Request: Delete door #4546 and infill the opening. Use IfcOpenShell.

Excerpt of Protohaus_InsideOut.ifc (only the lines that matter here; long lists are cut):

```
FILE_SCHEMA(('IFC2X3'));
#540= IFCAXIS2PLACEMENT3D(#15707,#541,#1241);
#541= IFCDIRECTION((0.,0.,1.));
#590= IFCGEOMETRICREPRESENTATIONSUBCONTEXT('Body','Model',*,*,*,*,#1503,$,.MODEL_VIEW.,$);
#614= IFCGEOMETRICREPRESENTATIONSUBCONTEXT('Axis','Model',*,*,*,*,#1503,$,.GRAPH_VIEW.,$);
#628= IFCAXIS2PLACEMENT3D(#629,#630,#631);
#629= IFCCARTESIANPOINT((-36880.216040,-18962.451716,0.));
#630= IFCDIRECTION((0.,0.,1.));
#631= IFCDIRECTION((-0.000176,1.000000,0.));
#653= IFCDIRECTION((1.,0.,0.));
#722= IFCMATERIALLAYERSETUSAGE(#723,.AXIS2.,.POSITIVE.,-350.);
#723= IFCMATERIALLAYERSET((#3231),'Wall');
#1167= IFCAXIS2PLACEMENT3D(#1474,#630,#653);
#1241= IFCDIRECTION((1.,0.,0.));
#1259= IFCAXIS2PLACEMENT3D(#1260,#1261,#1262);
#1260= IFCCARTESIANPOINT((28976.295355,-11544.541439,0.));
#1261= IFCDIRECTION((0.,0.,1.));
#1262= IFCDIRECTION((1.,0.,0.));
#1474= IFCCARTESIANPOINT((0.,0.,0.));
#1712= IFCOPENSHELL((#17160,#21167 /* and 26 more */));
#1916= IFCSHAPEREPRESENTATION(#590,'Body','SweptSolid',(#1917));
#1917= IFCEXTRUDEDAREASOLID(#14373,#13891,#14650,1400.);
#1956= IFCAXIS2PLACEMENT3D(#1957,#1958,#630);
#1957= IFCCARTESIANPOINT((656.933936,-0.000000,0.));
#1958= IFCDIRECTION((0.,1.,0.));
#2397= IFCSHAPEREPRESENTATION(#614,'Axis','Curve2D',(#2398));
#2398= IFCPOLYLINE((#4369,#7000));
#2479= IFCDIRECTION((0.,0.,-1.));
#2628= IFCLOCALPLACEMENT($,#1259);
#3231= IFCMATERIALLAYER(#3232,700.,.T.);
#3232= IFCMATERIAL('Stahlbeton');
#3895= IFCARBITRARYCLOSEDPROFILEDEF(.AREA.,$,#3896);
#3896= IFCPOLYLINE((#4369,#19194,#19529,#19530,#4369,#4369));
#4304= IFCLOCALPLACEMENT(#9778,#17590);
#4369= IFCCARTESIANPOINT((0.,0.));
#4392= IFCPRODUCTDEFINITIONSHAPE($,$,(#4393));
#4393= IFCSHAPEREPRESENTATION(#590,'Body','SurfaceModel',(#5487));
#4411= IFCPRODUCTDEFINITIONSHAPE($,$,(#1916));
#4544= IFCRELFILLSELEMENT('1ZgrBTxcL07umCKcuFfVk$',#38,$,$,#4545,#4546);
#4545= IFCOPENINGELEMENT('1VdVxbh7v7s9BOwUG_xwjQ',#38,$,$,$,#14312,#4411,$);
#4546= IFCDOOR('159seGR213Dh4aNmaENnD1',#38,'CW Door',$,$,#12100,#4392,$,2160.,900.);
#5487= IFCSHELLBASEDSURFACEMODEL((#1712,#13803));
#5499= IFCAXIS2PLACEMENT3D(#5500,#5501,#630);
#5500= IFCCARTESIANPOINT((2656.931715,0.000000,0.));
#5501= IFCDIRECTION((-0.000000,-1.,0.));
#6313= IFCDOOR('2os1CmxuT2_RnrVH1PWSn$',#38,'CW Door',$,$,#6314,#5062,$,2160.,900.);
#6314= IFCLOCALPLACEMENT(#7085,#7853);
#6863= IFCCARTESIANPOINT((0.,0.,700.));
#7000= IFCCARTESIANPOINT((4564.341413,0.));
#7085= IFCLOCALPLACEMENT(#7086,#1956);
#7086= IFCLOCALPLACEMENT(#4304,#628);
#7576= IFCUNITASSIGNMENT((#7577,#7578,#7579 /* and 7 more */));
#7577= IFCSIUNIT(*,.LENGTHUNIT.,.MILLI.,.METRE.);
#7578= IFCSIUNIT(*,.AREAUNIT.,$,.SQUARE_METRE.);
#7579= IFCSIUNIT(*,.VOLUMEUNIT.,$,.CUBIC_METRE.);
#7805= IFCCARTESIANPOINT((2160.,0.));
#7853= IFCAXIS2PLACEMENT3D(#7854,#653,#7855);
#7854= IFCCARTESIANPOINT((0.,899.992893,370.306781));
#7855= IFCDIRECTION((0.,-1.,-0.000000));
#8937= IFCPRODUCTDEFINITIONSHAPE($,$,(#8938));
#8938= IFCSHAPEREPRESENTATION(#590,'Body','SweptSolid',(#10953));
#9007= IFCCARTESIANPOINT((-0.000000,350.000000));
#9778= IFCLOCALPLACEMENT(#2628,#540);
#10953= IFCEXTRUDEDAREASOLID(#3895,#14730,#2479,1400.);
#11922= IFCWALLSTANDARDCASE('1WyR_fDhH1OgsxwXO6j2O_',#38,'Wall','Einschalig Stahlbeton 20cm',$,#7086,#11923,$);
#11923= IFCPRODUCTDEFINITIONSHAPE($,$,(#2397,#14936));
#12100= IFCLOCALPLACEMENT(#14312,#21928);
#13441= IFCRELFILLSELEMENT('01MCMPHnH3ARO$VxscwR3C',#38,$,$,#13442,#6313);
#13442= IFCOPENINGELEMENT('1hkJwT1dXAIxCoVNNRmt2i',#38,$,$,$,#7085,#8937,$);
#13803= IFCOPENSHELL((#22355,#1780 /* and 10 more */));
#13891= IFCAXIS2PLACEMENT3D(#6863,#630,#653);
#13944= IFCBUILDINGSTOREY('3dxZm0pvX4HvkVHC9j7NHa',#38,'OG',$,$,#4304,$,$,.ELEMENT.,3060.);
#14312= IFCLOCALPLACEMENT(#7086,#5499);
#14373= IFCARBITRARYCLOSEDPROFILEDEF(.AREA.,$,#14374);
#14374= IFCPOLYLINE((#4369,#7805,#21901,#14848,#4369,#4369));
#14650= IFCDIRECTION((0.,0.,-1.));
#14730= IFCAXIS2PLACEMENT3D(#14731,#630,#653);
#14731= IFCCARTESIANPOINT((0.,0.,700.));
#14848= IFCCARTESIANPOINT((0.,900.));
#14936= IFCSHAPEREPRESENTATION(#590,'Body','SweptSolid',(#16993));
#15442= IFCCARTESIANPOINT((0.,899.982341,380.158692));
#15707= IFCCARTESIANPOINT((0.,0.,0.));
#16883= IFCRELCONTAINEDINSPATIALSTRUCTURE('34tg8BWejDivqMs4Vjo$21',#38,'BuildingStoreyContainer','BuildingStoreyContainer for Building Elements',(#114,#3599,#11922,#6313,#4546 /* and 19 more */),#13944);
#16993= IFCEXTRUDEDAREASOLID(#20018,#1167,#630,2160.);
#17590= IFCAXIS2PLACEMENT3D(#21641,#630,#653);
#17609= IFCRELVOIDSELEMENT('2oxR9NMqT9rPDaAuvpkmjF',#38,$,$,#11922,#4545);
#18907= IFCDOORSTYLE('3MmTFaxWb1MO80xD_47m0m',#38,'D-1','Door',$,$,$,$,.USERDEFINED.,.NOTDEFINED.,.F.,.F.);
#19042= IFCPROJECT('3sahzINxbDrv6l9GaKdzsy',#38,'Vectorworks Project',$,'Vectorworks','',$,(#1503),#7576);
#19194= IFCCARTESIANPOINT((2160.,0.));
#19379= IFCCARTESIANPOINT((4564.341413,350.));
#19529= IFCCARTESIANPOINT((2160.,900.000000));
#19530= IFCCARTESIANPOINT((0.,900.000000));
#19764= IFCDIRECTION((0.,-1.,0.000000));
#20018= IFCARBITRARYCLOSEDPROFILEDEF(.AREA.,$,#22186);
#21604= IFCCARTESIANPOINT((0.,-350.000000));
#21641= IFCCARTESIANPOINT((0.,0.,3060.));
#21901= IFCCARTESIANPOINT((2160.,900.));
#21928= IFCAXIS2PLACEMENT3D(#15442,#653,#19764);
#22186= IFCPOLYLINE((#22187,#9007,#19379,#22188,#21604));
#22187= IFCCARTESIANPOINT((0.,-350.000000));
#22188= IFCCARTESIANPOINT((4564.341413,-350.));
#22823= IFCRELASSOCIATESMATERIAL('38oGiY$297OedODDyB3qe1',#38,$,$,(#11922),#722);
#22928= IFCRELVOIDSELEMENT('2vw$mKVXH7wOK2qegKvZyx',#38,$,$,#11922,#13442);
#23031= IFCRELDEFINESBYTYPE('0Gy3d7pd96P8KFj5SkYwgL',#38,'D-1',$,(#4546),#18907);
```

```python
import ifcopenshell
import ifcopenshell.api.feature
import ifcopenshell.api.root
import ifcopenshell.geom
import ifcopenshell.util.shape

model = ifcopenshell.open("Protohaus_InsideOut.ifc")
settings = ifcopenshell.geom.settings()


def volume(element):
    """Net volume in cubic metres, openings subtracted."""
    shape = ifcopenshell.geom.create_shape(settings, element)
    return ifcopenshell.util.shape.get_volume(shape.geometry)


door = model.by_guid("159seGR213Dh4aNmaENnD1")
opening = door.FillsVoids[0].RelatingOpeningElement
wall = opening.VoidsElements[0].RelatingBuildingElement
before = volume(wall)

ifcopenshell.api.root.remove_product(model, product=door)
ifcopenshell.api.feature.remove_feature(model, feature=opening)

after = volume(wall)

print(f"wall volume {before:.3f} -> {after:.3f} m3")

model.write("Protohaus_InsideOut_v2.ifc")
```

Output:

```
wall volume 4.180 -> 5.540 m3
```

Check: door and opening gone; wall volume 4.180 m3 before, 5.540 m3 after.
